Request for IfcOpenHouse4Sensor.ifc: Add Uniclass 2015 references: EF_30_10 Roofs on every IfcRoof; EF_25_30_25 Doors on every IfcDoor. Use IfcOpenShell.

First a look at what the model holds.

```python
import ifcopenshell

model = ifcopenshell.open("IfcOpenHouse4Sensor.ifc")
print(model.schema)
print("classifications:", [c.Name for c in model.by_type("IfcClassification")])
for ifc_class in ("IfcDoor", "IfcRoof", "IfcStair", "IfcWall", "IfcWindow"):
    print(ifc_class, len(model.by_type(ifc_class)))
```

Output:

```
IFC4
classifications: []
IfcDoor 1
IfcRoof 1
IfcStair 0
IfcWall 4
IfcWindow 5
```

```python
import ifcopenshell
import ifcopenshell.api.classification

model = ifcopenshell.open("IfcOpenHouse4Sensor.ifc")

system = ifcopenshell.api.classification.add_classification(model, classification="Uniclass 2015")

codes = {
    "IfcRoof": ("EF_30_10", "Roofs"),
    "IfcDoor": ("EF_25_30_25", "Doors"),
}
for ifc_class, (code, name) in codes.items():
    products = model.by_type(ifc_class)
    ifcopenshell.api.classification.add_reference(
        model, products=products, classification=system, identification=code, name=name
    )
    print(code, len(products))

model.write("IfcOpenHouse4Sensor-out.ifc")
```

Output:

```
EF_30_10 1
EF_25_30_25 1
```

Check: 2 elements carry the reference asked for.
